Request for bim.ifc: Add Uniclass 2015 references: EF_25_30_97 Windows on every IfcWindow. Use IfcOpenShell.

First a look at what the model holds.

```python
import ifcopenshell

model = ifcopenshell.open("bim.ifc")
print(model.schema)
print("classifications:", [c.Name for c in model.by_type("IfcClassification")])
for ifc_class in ("IfcDoor", "IfcRoof", "IfcStair", "IfcWall", "IfcWindow"):
    print(ifc_class, len(model.by_type(ifc_class)))
```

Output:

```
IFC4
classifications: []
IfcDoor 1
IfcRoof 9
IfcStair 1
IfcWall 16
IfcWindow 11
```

```python
import ifcopenshell
import ifcopenshell.api.classification

model = ifcopenshell.open("bim.ifc")

system = ifcopenshell.api.classification.add_classification(model, classification="Uniclass 2015")

codes = {
    "IfcWindow": ("EF_25_30_97", "Windows"),
}
for ifc_class, (code, name) in codes.items():
    products = model.by_type(ifc_class)
    ifcopenshell.api.classification.add_reference(
        model, products=products, classification=system, identification=code, name=name
    )
    print(code, len(products))

model.write("bim_edited.ifc")
```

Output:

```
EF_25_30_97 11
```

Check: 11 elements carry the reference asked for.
